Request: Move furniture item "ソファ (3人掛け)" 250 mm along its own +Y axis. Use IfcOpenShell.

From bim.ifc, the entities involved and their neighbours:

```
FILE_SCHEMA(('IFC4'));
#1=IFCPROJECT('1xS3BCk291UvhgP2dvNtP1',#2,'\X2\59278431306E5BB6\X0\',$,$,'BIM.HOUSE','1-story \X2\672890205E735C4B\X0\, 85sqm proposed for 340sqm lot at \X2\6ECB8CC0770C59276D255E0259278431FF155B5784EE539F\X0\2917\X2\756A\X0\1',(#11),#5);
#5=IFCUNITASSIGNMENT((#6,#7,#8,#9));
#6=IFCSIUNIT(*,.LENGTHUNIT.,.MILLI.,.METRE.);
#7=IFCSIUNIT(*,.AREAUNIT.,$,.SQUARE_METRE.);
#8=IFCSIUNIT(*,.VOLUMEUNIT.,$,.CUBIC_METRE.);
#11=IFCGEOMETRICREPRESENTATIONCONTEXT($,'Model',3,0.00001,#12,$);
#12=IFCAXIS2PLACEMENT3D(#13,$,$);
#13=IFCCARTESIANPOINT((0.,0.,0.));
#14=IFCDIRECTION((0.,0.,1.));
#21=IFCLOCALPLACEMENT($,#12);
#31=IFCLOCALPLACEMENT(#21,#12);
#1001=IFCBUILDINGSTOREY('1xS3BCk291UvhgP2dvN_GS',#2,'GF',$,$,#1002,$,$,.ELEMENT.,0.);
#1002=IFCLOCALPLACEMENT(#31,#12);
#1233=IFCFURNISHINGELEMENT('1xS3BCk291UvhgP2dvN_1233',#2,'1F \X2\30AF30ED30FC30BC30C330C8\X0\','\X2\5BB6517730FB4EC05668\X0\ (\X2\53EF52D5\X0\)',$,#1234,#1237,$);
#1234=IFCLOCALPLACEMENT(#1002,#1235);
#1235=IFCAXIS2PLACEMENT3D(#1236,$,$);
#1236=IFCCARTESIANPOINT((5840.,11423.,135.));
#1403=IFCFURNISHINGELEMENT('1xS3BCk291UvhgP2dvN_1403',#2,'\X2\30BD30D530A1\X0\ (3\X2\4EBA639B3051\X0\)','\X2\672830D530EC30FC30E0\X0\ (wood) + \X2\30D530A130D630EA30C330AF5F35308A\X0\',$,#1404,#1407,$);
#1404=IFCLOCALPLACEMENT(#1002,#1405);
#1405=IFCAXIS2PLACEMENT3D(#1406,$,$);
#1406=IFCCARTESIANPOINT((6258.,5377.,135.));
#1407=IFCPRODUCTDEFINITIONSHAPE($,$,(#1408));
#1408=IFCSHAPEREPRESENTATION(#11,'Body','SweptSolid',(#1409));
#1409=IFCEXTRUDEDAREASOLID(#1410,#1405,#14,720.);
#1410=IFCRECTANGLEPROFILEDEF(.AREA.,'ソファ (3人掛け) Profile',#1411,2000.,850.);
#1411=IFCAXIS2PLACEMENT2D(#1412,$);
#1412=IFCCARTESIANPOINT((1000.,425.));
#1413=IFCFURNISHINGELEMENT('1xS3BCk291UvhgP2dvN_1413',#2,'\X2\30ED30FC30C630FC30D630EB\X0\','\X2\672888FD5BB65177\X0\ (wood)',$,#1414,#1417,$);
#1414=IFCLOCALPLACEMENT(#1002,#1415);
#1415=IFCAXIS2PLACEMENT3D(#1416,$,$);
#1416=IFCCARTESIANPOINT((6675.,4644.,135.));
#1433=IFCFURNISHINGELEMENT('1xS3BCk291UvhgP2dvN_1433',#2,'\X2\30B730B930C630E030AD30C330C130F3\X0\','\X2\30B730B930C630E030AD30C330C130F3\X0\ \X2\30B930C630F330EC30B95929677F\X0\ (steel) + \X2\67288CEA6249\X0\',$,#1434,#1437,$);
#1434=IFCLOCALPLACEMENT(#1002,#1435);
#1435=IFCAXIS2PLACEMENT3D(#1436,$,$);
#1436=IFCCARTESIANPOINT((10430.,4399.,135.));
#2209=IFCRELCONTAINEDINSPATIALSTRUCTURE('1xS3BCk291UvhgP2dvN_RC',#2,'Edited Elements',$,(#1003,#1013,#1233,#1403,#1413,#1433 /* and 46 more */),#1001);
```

```python
import ifcopenshell
import ifcopenshell.api.geometry
import ifcopenshell.util.placement
import ifcopenshell.util.unit

model = ifcopenshell.open("bim.ifc")
unit_scale = ifcopenshell.util.unit.calculate_unit_scale(model)

item = model.by_guid("1xS3BCk291UvhgP2dvN_1403")
matrix = ifcopenshell.util.placement.get_local_placement(item.ObjectPlacement)
matrix[:3, 3] += matrix[:3, 1] * 0.25 / unit_scale
ifcopenshell.api.geometry.edit_object_placement(model, product=item, matrix=matrix, is_si=False)

print(ifcopenshell.util.placement.get_local_placement(item.ObjectPlacement).round(3) + 0.0)

model.write("bim_v2.ifc")
```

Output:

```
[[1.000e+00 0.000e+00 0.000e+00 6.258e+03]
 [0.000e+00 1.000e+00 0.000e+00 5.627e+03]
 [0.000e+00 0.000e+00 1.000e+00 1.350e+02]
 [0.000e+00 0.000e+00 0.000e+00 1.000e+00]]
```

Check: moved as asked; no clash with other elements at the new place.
